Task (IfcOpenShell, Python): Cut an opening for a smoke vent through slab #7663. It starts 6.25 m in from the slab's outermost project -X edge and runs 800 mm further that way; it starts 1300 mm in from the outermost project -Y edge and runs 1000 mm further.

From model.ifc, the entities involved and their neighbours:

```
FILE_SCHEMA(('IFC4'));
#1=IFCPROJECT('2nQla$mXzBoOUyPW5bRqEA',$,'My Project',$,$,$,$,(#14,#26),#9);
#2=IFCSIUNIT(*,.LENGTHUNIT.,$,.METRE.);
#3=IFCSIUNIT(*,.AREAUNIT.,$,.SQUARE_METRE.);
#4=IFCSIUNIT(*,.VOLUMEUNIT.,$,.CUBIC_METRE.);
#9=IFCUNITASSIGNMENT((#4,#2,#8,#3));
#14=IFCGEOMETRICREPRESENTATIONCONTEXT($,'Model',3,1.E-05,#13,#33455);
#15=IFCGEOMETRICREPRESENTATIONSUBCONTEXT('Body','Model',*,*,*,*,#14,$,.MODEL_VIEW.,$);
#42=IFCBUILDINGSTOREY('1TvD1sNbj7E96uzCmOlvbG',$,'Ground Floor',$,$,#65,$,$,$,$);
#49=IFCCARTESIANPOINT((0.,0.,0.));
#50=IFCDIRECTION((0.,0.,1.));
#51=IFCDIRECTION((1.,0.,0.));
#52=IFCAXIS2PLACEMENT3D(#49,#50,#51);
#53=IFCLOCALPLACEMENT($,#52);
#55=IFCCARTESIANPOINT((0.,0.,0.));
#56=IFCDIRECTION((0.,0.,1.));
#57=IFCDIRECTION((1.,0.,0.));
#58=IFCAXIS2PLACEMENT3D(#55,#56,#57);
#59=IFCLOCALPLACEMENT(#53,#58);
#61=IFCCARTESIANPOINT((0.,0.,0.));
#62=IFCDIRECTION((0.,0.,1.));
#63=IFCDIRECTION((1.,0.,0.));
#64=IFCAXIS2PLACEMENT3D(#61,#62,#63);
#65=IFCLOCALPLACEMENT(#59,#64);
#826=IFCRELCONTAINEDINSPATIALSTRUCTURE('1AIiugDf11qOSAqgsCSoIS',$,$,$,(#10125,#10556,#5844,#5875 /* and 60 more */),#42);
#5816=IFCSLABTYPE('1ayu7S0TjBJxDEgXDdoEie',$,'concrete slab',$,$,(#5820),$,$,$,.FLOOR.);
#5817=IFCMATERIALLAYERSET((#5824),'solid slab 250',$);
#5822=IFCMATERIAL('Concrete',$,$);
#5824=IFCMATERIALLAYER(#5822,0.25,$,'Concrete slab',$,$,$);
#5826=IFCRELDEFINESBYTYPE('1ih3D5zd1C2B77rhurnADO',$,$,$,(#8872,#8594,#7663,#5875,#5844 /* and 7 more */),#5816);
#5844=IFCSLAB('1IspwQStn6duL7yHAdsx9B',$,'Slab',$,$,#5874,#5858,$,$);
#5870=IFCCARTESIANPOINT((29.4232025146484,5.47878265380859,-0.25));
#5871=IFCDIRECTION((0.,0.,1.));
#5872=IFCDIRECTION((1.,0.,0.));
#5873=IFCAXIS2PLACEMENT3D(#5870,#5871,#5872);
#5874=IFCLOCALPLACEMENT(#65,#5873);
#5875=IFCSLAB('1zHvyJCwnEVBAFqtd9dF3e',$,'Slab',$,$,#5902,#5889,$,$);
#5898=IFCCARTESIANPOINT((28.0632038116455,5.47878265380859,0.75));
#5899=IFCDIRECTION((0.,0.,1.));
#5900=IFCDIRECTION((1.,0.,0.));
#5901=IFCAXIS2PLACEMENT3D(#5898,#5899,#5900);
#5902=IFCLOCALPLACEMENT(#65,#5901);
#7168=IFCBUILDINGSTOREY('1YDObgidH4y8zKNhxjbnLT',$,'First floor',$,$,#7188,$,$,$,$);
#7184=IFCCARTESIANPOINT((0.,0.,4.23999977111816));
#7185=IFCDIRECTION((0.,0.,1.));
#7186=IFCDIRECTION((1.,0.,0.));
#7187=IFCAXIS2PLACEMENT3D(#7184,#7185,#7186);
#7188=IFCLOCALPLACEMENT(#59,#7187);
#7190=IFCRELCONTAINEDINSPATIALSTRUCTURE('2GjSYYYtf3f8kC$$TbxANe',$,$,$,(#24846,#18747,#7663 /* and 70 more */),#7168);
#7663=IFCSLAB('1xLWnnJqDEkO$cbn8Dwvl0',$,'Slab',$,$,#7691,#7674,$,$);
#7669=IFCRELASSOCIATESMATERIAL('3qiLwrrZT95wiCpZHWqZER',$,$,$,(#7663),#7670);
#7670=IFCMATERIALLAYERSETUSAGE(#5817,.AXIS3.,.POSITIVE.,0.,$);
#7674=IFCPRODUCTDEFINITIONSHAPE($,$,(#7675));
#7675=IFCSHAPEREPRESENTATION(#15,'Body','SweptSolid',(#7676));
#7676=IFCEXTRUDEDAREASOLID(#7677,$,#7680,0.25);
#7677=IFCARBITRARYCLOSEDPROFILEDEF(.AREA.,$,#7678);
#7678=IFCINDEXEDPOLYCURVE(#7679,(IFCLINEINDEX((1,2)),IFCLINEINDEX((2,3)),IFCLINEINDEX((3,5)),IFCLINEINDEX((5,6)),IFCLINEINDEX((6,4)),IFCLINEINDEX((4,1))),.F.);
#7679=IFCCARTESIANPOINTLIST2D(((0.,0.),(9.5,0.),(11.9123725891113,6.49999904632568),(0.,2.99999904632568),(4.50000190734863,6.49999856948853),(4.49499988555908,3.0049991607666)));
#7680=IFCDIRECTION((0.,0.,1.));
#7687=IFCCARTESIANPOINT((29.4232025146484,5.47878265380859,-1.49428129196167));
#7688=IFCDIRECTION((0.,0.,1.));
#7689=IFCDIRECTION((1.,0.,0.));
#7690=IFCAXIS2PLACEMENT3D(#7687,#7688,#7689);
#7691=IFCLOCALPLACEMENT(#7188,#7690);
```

```python
import numpy as np
import ifcopenshell
import ifcopenshell.api.feature
import ifcopenshell.api.geometry
import ifcopenshell.api.root
import ifcopenshell.geom
import ifcopenshell.util.placement
import ifcopenshell.util.representation
import ifcopenshell.util.shape
import ifcopenshell.util.unit

model = ifcopenshell.open("model.ifc")
unit_scale = ifcopenshell.util.unit.calculate_unit_scale(model)
settings = ifcopenshell.geom.settings()


def volume(element):
    """Net volume in cubic metres, openings subtracted."""
    shape = ifcopenshell.geom.create_shape(settings, element)
    return ifcopenshell.util.shape.get_volume(shape.geometry)


slab = model.by_guid("1xLWnnJqDEkO$cbn8Dwvl0")
before = volume(slab)

# Extent in the slab's own axes, in metres. The edges named are its -X and -Y sides.
slab_shape = ifcopenshell.geom.create_shape(settings, slab)
vertices = ifcopenshell.util.shape.get_vertices(slab_shape.geometry)
x_min, y_min, bottom = vertices.min(axis=0)
top = vertices[:, 2].max()

opening = ifcopenshell.api.root.create_entity(model, ifc_class="IfcOpeningElement", name="Smoke vent opening", predefined_type="OPENING")
context = ifcopenshell.util.representation.get_context(model, "Model", "Body", "MODEL_VIEW")
width, depth = 0.8, 1
outline = [(0.0, 0.0), (width, 0.0), (width, depth), (0.0, depth), (0.0, 0.0)]
# Overshoot both faces by 50 mm so the cut is clean.
shape = ifcopenshell.api.geometry.add_slab_representation(
    model, context=context, depth=top - bottom + 0.1, polyline=outline
)
ifcopenshell.api.geometry.assign_representation(model, product=opening, representation=shape)

matrix = ifcopenshell.util.placement.get_local_placement(slab.ObjectPlacement)
matrix[:, 3] = matrix @ np.append(np.array([x_min + 6.25, y_min + 1.3, bottom - 0.05]) / unit_scale, 1.0)
ifcopenshell.api.geometry.edit_object_placement(model, product=opening, matrix=matrix, is_si=False)
ifcopenshell.api.feature.add_feature(model, feature=opening, element=slab)

after = volume(slab)

print(f"slab volume {before:.3f} -> {after:.3f} m3")

model.write("model_rev.ifc")
```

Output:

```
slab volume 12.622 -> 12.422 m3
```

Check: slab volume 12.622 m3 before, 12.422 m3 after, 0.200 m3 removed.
